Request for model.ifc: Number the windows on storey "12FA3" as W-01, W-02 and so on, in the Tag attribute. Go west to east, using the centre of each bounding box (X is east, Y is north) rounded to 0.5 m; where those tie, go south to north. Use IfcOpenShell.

First a look at what the model holds.

```python
import ifcopenshell
import ifcopenshell.util.element
import ifcopenshell.util.placement

model = ifcopenshell.open("model.ifc")
print(model.schema)
storey = next(s for s in model.by_type("IfcBuildingStorey") if s.Name == "12FA3")
windows = [e for e in ifcopenshell.util.element.get_decomposition(storey) if e.is_a("IfcWindow")]
for e in sorted(windows, key=lambda e: e.id()):
    origin = ifcopenshell.util.placement.get_local_placement(e.ObjectPlacement)[:3, 3]
    print(e.id(), e.Tag, e.Name, origin.round(2) + 0.0, sep=" | ")
```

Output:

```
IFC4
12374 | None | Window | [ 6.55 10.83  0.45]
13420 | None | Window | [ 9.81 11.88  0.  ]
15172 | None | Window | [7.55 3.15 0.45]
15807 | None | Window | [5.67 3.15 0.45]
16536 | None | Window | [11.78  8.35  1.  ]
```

```python
import ifcopenshell
import ifcopenshell.geom
import ifcopenshell.util.element
import ifcopenshell.util.shape

model = ifcopenshell.open("model.ifc")
settings = ifcopenshell.geom.settings()
settings.set("use-world-coords", True)


def centre(element):
    shape = ifcopenshell.geom.create_shape(settings, element)
    return ifcopenshell.util.shape.get_bbox_centroid(shape.geometry)


storey = next(s for s in model.by_type("IfcBuildingStorey") if s.Name == "12FA3")
windows = [e for e in ifcopenshell.util.element.get_decomposition(storey) if e.is_a("IfcWindow")]

# Insertion points can sit at a corner or the storey origin, so sort by the geometry (in metres).
centres = {e: centre(e) for e in windows}
windows.sort(key=lambda e: (round(centres[e][0] / 0.5), centres[e][1]))

for i, e in enumerate(windows, start=1):
    number = f"W-{i:02d}"
    e.Tag = number
    print(e.id(), number)

model.write("model_rev.ifc")
```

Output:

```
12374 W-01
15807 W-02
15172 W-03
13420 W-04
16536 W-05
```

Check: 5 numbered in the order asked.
